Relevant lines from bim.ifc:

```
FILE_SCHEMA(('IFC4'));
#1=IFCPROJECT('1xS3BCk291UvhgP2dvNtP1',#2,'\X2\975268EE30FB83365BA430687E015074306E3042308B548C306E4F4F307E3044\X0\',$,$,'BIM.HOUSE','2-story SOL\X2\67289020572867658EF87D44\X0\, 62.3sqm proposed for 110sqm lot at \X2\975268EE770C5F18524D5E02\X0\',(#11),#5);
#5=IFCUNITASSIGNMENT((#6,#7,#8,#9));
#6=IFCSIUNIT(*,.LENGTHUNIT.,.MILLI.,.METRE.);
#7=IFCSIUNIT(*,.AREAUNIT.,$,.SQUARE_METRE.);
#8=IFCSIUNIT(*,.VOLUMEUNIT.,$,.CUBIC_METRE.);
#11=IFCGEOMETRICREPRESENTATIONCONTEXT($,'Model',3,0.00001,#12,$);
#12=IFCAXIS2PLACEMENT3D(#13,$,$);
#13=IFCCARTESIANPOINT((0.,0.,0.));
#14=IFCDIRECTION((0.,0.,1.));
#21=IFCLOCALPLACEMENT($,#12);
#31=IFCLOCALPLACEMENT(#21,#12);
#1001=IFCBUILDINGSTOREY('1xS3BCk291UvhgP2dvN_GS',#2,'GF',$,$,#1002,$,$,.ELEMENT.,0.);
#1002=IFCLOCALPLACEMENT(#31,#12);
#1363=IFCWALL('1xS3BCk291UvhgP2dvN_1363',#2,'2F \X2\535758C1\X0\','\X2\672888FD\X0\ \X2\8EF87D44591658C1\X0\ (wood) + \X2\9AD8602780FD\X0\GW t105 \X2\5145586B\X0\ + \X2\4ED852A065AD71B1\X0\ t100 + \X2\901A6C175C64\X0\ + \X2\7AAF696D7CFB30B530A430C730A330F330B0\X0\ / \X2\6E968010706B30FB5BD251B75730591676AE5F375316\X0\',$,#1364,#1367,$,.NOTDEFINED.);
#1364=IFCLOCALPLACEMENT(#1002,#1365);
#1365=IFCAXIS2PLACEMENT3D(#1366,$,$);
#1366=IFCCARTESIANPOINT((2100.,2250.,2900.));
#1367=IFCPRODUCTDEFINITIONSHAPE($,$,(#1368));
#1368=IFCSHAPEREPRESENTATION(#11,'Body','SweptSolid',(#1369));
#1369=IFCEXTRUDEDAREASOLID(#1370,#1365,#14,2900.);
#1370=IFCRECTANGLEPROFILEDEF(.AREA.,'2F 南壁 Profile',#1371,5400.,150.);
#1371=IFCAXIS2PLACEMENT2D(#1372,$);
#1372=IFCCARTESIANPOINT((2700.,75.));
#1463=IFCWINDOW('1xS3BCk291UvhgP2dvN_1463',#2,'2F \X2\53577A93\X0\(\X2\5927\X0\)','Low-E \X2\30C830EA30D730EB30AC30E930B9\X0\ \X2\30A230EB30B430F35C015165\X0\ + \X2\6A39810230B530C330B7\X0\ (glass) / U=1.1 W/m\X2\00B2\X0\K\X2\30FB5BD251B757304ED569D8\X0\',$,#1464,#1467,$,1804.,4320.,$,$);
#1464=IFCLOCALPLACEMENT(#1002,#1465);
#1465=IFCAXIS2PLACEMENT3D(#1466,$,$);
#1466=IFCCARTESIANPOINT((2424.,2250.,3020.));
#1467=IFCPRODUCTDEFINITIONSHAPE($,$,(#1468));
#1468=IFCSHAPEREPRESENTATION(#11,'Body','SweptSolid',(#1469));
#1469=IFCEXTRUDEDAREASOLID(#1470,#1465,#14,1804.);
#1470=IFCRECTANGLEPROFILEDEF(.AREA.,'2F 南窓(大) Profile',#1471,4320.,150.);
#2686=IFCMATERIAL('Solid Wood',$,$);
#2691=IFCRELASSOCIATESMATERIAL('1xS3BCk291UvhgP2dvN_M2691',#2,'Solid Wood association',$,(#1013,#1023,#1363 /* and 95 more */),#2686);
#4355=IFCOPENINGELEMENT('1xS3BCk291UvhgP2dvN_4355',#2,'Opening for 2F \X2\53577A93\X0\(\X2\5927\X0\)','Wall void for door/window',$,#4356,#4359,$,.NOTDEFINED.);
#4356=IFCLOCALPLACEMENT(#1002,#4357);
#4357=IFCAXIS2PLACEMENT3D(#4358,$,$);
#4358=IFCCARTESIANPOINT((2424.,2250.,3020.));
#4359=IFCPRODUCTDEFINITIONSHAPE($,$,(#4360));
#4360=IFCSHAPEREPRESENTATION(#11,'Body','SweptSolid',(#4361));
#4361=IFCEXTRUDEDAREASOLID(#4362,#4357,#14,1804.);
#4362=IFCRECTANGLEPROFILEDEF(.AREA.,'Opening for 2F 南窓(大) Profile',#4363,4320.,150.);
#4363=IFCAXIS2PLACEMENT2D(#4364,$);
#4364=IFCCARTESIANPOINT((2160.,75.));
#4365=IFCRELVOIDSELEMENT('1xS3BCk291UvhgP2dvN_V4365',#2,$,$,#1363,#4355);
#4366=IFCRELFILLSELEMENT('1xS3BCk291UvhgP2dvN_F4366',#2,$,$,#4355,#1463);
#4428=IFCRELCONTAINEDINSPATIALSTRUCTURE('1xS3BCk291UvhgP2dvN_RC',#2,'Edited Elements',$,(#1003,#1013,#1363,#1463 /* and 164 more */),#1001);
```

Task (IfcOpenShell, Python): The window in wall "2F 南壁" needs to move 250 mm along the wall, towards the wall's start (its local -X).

```python
import ifcopenshell
import ifcopenshell.api.geometry
import ifcopenshell.util.placement
import ifcopenshell.util.unit

model = ifcopenshell.open("bim.ifc")
unit_scale = ifcopenshell.util.unit.calculate_unit_scale(model)

window = model.by_guid("1xS3BCk291UvhgP2dvN_1463")
opening = window.FillsVoids[0].RelatingOpeningElement
wall = opening.VoidsElements[0].RelatingBuildingElement

wall_matrix = ifcopenshell.util.placement.get_local_placement(wall.ObjectPlacement)
shift = wall_matrix[:3, 0] * -0.25 / unit_scale
before = ifcopenshell.util.placement.get_local_placement(window.ObjectPlacement)[:3, 3].copy()

# The window is not placed relative to its opening, so move both.
for product in (opening, window):
    matrix = ifcopenshell.util.placement.get_local_placement(product.ObjectPlacement)
    matrix[:3, 3] += shift
    ifcopenshell.api.geometry.edit_object_placement(model, product=product, matrix=matrix, is_si=False)

after = ifcopenshell.util.placement.get_local_placement(window.ObjectPlacement)[:3, 3]
print("window moved by", (after - before).round(3) + 0.0)

model.write("bim_rev.ifc")
```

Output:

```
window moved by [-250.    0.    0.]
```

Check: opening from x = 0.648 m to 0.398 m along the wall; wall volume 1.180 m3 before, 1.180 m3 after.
